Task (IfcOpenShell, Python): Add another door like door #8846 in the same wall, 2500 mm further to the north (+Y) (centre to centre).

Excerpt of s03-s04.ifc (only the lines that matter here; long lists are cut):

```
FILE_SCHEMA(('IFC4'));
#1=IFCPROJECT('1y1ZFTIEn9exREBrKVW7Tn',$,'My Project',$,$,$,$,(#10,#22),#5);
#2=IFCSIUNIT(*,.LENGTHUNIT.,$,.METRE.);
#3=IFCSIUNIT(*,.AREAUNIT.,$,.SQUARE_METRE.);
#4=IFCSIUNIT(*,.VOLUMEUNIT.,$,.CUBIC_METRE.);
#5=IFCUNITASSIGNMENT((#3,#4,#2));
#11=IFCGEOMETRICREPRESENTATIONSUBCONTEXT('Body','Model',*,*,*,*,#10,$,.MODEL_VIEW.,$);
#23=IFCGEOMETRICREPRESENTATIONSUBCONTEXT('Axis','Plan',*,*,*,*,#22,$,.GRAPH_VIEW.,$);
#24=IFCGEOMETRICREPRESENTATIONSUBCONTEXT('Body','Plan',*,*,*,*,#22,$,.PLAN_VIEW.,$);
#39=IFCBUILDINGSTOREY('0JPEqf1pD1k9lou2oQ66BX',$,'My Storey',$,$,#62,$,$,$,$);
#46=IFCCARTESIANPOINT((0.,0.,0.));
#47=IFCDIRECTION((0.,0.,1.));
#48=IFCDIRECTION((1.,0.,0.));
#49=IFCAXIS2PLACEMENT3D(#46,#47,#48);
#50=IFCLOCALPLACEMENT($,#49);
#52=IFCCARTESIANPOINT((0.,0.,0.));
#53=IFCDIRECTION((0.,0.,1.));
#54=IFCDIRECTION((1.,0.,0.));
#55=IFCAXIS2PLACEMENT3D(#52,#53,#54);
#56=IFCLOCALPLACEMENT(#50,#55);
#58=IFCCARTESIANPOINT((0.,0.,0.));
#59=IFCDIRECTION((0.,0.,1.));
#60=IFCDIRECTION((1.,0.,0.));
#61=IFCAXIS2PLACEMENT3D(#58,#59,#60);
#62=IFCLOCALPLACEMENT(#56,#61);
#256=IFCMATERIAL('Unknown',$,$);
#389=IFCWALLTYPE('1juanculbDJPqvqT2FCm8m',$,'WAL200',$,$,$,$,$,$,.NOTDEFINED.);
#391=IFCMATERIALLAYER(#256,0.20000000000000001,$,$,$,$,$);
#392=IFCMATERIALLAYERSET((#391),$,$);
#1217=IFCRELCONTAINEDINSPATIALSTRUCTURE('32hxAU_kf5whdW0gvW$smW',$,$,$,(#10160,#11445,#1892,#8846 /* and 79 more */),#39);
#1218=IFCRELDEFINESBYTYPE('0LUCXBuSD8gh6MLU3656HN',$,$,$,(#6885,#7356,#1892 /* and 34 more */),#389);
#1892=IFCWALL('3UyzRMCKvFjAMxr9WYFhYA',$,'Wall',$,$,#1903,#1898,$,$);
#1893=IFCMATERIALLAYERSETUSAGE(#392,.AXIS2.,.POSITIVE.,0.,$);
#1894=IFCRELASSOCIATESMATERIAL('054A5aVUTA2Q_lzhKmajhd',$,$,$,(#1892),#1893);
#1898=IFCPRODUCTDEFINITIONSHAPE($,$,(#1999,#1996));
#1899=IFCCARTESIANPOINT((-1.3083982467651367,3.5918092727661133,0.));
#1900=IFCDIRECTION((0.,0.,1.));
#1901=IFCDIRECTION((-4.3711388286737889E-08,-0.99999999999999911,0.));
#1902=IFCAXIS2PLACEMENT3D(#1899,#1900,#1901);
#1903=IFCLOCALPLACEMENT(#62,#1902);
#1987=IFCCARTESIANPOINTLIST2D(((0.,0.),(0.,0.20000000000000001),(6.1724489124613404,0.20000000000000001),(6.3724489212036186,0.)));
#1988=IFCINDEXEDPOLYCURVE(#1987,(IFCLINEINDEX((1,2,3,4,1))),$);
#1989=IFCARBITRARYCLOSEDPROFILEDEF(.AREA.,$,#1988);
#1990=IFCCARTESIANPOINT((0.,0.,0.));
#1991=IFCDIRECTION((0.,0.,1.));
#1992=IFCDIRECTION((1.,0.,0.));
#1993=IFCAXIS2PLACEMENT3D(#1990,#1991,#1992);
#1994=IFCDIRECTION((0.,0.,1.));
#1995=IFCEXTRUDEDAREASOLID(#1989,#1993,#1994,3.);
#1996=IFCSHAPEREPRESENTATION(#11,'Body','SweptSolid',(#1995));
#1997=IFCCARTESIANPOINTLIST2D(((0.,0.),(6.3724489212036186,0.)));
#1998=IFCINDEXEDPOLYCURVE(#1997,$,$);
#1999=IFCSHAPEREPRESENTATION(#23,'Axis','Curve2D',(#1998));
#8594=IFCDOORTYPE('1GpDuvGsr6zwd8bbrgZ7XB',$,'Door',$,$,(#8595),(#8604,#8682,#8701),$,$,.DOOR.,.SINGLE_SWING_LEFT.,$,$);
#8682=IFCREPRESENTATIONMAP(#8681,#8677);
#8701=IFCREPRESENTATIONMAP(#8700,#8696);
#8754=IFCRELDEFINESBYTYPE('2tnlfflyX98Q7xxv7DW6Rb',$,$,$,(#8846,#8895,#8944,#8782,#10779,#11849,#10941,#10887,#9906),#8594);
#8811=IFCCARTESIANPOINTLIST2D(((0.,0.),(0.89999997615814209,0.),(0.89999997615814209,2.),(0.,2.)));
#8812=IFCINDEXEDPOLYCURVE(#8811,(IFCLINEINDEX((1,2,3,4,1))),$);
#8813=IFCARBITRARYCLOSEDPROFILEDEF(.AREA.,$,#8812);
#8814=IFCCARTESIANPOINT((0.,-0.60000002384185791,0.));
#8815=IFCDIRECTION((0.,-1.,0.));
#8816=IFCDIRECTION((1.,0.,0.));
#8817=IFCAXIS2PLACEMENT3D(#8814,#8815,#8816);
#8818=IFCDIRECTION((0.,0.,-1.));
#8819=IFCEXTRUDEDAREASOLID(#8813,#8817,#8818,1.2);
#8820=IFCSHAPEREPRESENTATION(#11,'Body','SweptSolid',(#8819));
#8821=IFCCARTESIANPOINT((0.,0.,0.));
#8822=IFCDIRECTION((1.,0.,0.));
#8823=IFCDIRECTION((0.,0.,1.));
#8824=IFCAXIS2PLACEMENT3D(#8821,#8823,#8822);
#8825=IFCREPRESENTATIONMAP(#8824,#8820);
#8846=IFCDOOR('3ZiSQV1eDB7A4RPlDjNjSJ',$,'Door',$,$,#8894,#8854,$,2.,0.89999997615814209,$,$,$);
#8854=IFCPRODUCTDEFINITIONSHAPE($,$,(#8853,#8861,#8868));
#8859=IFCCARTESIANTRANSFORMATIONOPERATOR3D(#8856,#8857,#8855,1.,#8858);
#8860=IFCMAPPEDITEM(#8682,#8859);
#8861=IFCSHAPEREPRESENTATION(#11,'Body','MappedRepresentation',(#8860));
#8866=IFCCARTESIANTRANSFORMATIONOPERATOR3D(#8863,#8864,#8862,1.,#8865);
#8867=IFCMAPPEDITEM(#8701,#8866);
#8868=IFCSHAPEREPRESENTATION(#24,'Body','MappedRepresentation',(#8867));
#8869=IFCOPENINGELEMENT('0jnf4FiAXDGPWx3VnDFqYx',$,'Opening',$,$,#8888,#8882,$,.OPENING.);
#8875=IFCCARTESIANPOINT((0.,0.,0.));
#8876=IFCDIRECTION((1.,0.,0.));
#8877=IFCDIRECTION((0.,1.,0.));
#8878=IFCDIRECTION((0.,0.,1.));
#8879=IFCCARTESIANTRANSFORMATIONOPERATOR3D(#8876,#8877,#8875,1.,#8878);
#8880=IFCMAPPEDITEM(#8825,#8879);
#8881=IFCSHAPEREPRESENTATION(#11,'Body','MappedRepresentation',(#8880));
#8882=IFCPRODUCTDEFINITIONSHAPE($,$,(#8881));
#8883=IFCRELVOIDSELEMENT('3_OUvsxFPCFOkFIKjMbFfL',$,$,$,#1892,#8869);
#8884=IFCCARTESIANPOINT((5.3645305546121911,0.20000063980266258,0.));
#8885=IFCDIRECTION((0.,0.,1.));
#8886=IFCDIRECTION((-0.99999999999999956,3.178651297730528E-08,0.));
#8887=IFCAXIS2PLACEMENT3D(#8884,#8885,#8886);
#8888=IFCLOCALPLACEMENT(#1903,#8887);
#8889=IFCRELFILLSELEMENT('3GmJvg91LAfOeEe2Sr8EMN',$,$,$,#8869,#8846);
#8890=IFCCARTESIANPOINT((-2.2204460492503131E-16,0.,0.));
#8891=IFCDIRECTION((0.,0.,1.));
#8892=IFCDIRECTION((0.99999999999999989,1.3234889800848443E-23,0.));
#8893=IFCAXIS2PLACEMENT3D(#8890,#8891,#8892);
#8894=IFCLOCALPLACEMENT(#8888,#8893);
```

```python
import ifcopenshell
import ifcopenshell.api.feature
import ifcopenshell.api.geometry
import ifcopenshell.api.root
import ifcopenshell.geom
import ifcopenshell.util.element
import ifcopenshell.util.placement
import ifcopenshell.util.shape
import ifcopenshell.util.unit

model = ifcopenshell.open("s03-s04.ifc")
unit_scale = ifcopenshell.util.unit.calculate_unit_scale(model)
settings = ifcopenshell.geom.settings()


def volume(element):
    """Net volume in cubic metres, openings subtracted."""
    shape = ifcopenshell.geom.create_shape(settings, element)
    return ifcopenshell.util.shape.get_volume(shape.geometry)


door = model.by_guid("3ZiSQV1eDB7A4RPlDjNjSJ")
opening = door.FillsVoids[0].RelatingOpeningElement
wall = opening.VoidsElements[0].RelatingBuildingElement
before = volume(wall)
shift = ifcopenshell.util.placement.get_local_placement(wall.ObjectPlacement)[:3, 0] * -2.5 / unit_scale

# copy_class copies the void relationship, type, container and properties, but no geometry.
new_opening = ifcopenshell.api.root.copy_class(model, product=opening)
new_opening.Representation = ifcopenshell.util.element.copy_deep(
    model, opening.Representation, exclude=["IfcGeometricRepresentationContext", "IfcRepresentationMap"]
)
new_door = ifcopenshell.api.root.copy_class(model, product=door)
new_door.Representation = ifcopenshell.util.element.copy_deep(
    model, door.Representation, exclude=["IfcGeometricRepresentationContext", "IfcRepresentationMap"]
)
ifcopenshell.api.feature.add_filling(model, opening=new_opening, element=new_door)

for old, new in ((opening, new_opening), (door, new_door)):
    matrix = ifcopenshell.util.placement.get_local_placement(old.ObjectPlacement)
    matrix[:3, 3] += shift
    ifcopenshell.api.geometry.edit_object_placement(model, product=new, matrix=matrix, is_si=False)

after = volume(wall)

print(f"wall volume {before:.3f} -> {after:.3f} m3")

model.write("s03-s04_updated.ifc")
```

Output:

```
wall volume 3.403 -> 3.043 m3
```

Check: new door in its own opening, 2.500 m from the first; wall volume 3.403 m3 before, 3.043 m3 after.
